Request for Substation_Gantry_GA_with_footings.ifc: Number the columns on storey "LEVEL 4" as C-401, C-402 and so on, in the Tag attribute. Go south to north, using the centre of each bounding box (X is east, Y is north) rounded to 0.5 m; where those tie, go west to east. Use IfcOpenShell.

First a look at what the model holds.

```python
import ifcopenshell
import ifcopenshell.util.element
import ifcopenshell.util.placement

model = ifcopenshell.open("Substation_Gantry_GA_with_footings.ifc")
print(model.schema)
storey = next(s for s in model.by_type("IfcBuildingStorey") if s.Name == "LEVEL 4")
columns = [e for e in ifcopenshell.util.element.get_decomposition(storey) if e.is_a("IfcColumn")]
for e in sorted(columns, key=lambda e: e.id()):
    origin = ifcopenshell.util.placement.get_local_placement(e.ObjectPlacement)[:3, 3]
    print(e.id(), e.Tag, e.Name, origin.round(2) + 0.0, sep=" | ")
```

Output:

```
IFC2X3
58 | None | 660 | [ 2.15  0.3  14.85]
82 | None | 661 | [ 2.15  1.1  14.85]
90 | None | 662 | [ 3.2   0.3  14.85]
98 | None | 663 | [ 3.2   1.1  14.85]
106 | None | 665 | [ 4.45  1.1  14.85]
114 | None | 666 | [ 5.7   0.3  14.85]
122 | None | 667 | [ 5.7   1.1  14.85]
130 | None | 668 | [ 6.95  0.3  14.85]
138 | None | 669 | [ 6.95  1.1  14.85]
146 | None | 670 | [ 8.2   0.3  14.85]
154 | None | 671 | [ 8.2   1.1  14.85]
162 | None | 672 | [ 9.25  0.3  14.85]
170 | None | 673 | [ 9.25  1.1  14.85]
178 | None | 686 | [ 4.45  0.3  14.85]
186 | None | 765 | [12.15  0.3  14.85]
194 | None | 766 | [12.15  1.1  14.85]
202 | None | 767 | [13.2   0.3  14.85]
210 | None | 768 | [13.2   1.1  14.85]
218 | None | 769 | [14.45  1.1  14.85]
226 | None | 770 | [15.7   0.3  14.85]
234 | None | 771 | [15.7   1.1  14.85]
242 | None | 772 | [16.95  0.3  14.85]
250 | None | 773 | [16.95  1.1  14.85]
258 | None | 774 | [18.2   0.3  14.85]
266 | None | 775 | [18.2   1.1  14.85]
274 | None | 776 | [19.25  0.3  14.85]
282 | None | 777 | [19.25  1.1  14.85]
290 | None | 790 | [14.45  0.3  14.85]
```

```python
import ifcopenshell
import ifcopenshell.geom
import ifcopenshell.util.element
import ifcopenshell.util.shape

model = ifcopenshell.open("Substation_Gantry_GA_with_footings.ifc")
settings = ifcopenshell.geom.settings()
settings.set("use-world-coords", True)


def centre(element):
    shape = ifcopenshell.geom.create_shape(settings, element)
    return ifcopenshell.util.shape.get_bbox_centroid(shape.geometry)


storey = next(s for s in model.by_type("IfcBuildingStorey") if s.Name == "LEVEL 4")
columns = [e for e in ifcopenshell.util.element.get_decomposition(storey) if e.is_a("IfcColumn")]

# Insertion points can sit at a corner or the storey origin, so sort by the geometry (in metres).
centres = {e: centre(e) for e in columns}
columns.sort(key=lambda e: (round(centres[e][1] / 0.5), centres[e][0]))

for i, e in enumerate(columns, start=1):
    number = f"C-4{i:02d}"
    e.Tag = number
    print(e.id(), number)

model.write("Substation_Gantry_GA_with_footings-out.ifc")
```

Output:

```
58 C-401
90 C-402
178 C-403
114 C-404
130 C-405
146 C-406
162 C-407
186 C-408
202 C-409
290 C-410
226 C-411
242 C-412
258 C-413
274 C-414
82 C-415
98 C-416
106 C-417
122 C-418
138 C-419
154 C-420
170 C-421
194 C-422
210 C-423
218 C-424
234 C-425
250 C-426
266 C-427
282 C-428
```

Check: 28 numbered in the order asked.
